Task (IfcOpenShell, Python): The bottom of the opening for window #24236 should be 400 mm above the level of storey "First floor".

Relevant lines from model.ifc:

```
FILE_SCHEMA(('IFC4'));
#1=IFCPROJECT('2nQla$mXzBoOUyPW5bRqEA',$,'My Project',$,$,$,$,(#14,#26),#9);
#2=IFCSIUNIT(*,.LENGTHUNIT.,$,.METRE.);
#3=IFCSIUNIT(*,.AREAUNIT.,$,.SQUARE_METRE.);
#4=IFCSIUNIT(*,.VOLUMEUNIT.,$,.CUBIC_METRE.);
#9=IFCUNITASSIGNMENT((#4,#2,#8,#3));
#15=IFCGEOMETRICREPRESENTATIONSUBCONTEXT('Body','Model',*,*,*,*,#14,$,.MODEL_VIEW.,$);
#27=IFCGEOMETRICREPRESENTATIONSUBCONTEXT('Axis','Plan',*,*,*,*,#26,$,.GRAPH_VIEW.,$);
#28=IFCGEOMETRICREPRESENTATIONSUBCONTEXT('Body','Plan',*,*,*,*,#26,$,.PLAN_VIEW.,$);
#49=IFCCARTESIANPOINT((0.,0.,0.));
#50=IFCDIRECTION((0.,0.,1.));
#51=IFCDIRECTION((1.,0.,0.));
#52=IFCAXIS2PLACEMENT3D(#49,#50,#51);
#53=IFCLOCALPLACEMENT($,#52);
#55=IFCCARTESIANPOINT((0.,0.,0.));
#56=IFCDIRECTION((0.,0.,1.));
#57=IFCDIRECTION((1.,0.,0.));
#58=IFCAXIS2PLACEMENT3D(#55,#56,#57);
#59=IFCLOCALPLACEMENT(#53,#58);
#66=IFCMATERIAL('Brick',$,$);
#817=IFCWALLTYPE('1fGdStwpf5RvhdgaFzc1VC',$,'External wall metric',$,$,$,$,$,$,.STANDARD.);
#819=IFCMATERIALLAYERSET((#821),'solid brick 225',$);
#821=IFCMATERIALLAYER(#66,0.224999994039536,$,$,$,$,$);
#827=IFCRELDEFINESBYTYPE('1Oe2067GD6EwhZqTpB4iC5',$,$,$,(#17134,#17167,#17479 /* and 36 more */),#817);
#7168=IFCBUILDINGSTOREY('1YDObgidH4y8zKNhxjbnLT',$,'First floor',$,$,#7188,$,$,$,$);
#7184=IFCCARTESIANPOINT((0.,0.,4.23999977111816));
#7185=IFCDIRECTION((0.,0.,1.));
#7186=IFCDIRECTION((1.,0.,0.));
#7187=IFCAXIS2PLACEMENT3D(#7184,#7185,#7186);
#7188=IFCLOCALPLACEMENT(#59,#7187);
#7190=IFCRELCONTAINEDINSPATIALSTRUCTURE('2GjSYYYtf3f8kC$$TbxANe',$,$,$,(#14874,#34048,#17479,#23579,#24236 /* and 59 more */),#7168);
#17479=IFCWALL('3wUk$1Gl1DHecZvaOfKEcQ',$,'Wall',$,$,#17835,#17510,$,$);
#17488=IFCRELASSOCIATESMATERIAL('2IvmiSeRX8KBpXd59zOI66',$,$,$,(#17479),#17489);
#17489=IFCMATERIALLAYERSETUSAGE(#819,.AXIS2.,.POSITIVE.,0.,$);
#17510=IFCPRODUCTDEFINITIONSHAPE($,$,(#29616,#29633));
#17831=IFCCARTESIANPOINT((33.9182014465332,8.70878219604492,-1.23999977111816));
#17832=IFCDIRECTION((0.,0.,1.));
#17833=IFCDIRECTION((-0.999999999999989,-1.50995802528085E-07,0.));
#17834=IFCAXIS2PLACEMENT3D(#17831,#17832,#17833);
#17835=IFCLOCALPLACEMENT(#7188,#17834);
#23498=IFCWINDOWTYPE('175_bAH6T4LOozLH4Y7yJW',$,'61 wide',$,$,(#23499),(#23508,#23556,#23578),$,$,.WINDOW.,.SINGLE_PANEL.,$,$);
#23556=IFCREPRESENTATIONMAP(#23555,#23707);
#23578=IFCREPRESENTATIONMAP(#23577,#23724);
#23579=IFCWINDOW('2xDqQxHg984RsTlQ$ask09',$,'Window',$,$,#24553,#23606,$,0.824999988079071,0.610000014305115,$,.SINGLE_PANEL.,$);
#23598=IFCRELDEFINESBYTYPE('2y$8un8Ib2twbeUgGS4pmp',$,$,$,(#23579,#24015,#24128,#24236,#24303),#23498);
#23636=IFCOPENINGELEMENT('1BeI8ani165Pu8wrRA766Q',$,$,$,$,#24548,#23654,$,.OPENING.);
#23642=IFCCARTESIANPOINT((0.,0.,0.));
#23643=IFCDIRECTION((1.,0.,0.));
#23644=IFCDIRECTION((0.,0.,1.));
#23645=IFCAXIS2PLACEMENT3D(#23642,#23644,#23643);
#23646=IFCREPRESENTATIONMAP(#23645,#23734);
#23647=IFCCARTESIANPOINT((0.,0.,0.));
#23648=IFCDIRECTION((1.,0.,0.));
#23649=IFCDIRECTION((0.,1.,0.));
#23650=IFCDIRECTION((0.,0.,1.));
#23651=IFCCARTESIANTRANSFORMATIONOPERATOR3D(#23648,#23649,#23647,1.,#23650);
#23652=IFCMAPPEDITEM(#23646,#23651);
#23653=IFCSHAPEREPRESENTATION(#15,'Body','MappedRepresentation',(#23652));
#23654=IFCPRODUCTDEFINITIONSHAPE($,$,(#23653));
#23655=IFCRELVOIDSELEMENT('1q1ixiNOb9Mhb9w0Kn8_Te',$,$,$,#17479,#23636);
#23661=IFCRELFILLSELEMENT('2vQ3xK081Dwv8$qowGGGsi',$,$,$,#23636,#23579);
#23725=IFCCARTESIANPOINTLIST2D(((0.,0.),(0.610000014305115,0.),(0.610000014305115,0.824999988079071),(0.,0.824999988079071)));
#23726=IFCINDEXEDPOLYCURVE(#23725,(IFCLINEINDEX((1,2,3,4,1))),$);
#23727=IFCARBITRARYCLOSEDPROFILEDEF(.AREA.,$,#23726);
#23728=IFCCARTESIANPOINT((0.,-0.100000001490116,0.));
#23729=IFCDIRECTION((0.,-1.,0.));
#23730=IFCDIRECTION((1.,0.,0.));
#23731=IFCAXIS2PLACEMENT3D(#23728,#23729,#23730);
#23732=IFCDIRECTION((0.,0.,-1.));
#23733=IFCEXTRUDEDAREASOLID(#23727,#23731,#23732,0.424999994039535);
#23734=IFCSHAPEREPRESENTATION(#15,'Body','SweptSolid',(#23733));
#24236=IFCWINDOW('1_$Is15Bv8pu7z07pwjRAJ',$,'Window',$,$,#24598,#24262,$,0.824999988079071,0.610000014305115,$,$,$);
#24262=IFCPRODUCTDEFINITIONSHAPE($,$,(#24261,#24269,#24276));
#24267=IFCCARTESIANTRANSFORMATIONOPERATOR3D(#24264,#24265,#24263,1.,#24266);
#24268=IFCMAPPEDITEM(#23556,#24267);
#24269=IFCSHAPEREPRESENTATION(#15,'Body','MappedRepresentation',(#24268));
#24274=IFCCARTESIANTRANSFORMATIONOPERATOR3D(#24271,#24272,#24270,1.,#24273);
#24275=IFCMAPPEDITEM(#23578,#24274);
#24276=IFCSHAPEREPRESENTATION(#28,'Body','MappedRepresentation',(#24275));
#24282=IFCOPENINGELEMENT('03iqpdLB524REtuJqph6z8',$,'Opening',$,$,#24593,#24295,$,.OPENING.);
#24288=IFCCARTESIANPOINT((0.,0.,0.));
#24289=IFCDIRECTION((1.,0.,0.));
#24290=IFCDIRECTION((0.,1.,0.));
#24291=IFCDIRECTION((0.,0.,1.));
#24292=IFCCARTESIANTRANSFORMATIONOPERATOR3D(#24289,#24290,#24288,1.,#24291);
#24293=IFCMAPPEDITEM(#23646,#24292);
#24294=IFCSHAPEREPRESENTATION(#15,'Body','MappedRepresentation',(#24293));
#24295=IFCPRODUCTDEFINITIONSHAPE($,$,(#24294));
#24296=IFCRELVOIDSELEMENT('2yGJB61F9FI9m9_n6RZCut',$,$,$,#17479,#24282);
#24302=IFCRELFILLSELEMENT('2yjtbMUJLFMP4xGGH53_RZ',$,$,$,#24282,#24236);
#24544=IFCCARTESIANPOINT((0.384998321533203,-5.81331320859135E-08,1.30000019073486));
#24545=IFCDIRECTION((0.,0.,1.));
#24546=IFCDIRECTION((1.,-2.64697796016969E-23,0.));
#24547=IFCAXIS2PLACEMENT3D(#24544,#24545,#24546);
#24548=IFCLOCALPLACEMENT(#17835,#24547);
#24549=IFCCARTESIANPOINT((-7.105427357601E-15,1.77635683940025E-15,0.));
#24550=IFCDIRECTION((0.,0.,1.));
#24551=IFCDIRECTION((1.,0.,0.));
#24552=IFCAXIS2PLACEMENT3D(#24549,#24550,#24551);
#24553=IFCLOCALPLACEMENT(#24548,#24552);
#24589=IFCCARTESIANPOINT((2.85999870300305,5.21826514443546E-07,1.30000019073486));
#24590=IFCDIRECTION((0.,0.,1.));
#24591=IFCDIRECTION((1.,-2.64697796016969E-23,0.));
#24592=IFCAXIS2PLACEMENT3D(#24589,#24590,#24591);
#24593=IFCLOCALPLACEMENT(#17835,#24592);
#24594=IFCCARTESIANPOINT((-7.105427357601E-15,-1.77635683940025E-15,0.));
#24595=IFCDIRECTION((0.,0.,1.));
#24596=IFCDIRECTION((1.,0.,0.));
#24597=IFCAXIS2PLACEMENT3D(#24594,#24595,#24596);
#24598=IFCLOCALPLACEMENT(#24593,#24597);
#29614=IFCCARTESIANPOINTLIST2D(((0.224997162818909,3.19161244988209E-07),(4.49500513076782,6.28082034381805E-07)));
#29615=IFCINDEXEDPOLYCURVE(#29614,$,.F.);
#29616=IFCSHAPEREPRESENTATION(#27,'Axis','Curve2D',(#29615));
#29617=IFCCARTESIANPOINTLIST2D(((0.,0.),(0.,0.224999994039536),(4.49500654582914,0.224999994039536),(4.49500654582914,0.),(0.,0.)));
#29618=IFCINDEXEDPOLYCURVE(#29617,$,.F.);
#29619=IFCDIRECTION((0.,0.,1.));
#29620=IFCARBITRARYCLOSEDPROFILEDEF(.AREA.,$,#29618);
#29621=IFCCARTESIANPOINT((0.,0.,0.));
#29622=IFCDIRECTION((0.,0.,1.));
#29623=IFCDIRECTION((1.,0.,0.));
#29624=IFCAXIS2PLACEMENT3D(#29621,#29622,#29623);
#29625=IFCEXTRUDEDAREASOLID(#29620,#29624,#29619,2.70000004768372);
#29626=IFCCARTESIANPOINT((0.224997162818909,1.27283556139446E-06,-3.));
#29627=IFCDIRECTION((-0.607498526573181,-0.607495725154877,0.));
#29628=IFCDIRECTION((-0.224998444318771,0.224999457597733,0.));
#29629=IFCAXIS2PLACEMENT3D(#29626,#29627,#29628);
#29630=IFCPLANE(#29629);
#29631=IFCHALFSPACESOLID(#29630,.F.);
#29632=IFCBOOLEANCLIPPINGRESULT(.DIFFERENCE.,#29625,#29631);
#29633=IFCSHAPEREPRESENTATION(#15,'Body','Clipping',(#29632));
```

```python
import numpy as np
import ifcopenshell
import ifcopenshell.api.geometry
import ifcopenshell.geom
import ifcopenshell.util.element
import ifcopenshell.util.placement
import ifcopenshell.util.shape
import ifcopenshell.util.unit

model = ifcopenshell.open("model.ifc")
unit_scale = ifcopenshell.util.unit.calculate_unit_scale(model)

window = model.by_guid("1_$Is15Bv8pu7z07pwjRAJ")
opening = window.FillsVoids[0].RelatingOpeningElement
storey = ifcopenshell.util.element.get_container(window, ifc_class="IfcBuildingStorey")
level = ifcopenshell.util.placement.get_local_placement(storey.ObjectPlacement)[2, 3]

# The opening's origin need not be at the sill, so measure its lowest point.
shape = ifcopenshell.geom.create_shape(ifcopenshell.geom.settings(), opening)
bottom = ifcopenshell.util.shape.get_shape_bottom_elevation(shape, shape.geometry) / unit_scale
dz = level + 0.4 / unit_scale - bottom

shift = np.array([0.0, 0.0, dz])
# The window is placed relative to its opening, so it follows when the opening moves.
matrix = ifcopenshell.util.placement.get_local_placement(opening.ObjectPlacement)
matrix[:3, 3] += shift
ifcopenshell.api.geometry.edit_object_placement(
    model, product=opening, matrix=matrix, is_si=False, should_transform_children=True
)

print(f"moved by {dz * unit_scale:+.3f} m")

model.write("model_edited.ifc")
```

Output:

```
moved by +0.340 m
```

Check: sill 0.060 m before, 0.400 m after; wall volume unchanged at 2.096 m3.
